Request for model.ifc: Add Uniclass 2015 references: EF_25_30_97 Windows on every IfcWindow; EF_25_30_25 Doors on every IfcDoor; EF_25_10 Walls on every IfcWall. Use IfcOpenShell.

First a look at what the model holds.

```python
import ifcopenshell

model = ifcopenshell.open("model.ifc")
print(model.schema)
print("classifications:", [c.Name for c in model.by_type("IfcClassification")])
for ifc_class in ("IfcDoor", "IfcRoof", "IfcStair", "IfcWall", "IfcWindow"):
    print(ifc_class, len(model.by_type(ifc_class)))
```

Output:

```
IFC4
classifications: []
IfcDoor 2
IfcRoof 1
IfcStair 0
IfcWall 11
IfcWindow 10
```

```python
import ifcopenshell
import ifcopenshell.api.classification

model = ifcopenshell.open("model.ifc")

system = ifcopenshell.api.classification.add_classification(model, classification="Uniclass 2015")

codes = {
    "IfcWindow": ("EF_25_30_97", "Windows"),
    "IfcDoor": ("EF_25_30_25", "Doors"),
    "IfcWall": ("EF_25_10", "Walls"),
}
for ifc_class, (code, name) in codes.items():
    products = model.by_type(ifc_class)
    ifcopenshell.api.classification.add_reference(
        model, products=products, classification=system, identification=code, name=name
    )
    print(code, len(products))

model.write("model_updated.ifc")
```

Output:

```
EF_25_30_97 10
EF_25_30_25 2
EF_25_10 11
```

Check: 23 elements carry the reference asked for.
